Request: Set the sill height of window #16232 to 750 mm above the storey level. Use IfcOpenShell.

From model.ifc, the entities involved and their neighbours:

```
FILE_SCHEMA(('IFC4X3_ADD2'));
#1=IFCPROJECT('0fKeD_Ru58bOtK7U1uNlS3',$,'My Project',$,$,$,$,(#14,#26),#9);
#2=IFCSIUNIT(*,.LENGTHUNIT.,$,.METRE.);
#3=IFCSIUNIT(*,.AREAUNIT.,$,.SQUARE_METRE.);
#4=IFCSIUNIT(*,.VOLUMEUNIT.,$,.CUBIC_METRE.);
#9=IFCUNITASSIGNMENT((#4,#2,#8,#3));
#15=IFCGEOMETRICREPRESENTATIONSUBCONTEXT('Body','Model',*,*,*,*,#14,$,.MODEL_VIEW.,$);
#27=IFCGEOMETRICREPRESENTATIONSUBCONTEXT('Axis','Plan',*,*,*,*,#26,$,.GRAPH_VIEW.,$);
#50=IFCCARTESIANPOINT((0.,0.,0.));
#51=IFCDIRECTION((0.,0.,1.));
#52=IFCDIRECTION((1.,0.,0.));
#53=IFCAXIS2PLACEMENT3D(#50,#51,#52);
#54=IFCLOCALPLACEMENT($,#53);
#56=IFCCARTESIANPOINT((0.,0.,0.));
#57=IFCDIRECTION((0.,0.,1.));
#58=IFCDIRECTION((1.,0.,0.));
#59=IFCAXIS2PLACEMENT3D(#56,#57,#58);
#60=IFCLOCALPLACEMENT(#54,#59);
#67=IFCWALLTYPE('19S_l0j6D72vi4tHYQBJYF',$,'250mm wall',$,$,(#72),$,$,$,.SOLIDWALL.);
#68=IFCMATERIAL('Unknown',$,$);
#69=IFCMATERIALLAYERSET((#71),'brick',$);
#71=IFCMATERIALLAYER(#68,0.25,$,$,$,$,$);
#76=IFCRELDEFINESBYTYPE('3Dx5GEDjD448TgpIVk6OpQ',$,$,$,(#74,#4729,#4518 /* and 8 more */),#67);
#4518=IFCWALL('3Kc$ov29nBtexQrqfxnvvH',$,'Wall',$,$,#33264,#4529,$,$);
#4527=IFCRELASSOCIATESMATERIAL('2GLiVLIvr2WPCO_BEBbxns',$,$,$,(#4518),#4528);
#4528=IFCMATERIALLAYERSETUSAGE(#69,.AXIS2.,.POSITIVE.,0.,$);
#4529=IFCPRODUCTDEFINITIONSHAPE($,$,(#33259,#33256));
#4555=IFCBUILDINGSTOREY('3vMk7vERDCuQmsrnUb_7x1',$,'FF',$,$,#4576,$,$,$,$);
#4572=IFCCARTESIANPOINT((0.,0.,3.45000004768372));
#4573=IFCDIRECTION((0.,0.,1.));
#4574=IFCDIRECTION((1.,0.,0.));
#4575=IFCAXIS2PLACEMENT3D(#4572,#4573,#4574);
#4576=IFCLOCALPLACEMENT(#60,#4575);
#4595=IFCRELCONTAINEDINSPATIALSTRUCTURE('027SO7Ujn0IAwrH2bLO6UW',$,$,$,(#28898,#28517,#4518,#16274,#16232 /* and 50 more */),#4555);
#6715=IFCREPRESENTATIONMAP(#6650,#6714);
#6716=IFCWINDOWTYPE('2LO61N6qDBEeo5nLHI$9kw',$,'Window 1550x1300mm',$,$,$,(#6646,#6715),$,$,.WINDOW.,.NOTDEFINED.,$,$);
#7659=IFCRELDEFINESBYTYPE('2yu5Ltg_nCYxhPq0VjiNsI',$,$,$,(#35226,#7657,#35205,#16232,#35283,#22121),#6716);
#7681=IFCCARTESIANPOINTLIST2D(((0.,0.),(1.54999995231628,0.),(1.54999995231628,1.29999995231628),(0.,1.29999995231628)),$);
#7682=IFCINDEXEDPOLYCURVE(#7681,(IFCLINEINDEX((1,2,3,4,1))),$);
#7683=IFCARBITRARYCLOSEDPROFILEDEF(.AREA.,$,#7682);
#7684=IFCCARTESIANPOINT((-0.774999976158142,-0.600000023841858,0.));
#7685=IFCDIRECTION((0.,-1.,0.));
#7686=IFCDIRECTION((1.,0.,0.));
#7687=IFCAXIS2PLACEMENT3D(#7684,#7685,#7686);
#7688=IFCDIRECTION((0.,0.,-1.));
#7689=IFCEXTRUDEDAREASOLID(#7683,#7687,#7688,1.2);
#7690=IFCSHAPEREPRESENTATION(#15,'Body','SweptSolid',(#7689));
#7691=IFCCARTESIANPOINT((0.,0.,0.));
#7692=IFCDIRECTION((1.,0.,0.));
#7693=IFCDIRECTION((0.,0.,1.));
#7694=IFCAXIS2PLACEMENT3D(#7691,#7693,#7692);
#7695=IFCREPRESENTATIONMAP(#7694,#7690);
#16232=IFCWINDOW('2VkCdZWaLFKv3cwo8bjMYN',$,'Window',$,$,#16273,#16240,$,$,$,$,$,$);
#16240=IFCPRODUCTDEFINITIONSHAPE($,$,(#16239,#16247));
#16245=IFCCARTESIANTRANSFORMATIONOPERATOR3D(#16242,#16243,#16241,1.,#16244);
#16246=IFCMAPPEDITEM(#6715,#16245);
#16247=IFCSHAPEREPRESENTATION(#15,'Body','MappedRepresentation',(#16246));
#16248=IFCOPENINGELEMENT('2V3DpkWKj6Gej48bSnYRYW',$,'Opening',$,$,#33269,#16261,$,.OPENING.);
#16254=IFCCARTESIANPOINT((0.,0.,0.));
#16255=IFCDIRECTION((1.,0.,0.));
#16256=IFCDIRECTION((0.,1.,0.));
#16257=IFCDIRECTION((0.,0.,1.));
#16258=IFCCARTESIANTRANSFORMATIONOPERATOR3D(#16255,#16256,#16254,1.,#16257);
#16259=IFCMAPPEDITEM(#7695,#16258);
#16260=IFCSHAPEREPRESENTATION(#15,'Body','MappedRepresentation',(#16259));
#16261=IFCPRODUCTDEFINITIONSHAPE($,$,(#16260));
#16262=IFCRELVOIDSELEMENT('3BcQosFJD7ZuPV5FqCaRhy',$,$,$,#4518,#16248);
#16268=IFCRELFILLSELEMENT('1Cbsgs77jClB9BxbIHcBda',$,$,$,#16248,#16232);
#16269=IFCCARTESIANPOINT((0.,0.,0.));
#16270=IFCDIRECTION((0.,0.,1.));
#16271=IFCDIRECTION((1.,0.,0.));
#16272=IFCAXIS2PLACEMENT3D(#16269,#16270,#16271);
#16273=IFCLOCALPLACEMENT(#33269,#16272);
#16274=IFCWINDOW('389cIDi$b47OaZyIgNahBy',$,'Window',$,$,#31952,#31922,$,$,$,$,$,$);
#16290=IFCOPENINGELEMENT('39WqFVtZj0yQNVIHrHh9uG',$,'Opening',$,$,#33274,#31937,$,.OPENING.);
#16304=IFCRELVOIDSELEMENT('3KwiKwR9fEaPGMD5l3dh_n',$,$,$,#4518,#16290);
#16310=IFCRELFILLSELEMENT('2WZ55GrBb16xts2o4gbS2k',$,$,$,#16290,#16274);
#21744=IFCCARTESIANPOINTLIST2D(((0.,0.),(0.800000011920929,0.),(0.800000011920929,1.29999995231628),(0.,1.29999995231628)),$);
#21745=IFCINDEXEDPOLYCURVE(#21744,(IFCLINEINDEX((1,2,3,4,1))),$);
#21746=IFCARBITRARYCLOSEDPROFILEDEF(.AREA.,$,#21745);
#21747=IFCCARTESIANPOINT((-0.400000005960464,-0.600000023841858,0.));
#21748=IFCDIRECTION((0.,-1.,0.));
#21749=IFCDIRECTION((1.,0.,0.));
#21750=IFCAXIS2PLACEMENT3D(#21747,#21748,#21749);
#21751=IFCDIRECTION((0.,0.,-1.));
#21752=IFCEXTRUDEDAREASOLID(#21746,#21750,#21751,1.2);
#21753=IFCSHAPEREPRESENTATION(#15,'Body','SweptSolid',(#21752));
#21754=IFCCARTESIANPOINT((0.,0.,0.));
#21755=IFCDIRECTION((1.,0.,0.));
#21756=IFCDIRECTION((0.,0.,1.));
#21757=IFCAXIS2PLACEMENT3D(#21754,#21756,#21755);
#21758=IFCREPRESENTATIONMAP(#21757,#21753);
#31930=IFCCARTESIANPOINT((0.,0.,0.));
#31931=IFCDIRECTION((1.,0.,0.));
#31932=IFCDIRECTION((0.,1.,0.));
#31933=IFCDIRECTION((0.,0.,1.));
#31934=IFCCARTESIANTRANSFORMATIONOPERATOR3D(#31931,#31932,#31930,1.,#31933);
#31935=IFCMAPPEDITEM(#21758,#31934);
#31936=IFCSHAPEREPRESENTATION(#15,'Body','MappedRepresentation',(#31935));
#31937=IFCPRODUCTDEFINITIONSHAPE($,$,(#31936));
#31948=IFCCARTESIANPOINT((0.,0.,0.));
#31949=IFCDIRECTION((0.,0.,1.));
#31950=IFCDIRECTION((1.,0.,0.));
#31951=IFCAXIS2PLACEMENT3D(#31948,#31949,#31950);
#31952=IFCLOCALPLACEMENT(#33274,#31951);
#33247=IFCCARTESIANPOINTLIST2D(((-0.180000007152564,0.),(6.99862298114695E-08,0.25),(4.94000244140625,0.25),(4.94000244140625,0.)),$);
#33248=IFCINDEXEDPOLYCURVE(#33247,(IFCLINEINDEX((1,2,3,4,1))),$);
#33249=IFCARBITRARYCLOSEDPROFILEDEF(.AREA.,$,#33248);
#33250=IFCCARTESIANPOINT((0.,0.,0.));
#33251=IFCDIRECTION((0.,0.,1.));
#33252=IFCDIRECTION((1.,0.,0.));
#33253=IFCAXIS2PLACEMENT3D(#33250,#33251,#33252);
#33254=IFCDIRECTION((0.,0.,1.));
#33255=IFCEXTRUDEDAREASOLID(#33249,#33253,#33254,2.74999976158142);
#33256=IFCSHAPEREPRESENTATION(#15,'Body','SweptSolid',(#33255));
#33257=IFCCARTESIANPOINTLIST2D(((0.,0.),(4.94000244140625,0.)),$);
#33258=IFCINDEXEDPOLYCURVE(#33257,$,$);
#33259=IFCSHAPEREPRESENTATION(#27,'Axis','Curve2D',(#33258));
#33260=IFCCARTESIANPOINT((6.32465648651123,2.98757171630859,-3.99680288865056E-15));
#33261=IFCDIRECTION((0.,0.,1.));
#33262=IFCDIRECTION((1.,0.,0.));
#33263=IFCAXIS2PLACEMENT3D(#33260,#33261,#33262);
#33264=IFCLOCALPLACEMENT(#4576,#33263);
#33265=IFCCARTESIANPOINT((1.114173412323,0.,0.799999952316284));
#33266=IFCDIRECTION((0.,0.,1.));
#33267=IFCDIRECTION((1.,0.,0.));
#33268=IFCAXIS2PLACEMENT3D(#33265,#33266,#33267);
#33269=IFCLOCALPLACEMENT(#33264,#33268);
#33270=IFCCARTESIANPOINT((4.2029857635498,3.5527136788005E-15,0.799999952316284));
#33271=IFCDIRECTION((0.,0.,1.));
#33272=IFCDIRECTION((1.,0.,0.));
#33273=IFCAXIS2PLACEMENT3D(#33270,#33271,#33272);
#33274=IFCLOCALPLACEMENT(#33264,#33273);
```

```python
import numpy as np
import ifcopenshell
import ifcopenshell.api.geometry
import ifcopenshell.geom
import ifcopenshell.util.element
import ifcopenshell.util.placement
import ifcopenshell.util.shape
import ifcopenshell.util.unit

model = ifcopenshell.open("model.ifc")
unit_scale = ifcopenshell.util.unit.calculate_unit_scale(model)

window = model.by_guid("2VkCdZWaLFKv3cwo8bjMYN")
opening = window.FillsVoids[0].RelatingOpeningElement
storey = ifcopenshell.util.element.get_container(window, ifc_class="IfcBuildingStorey")
level = ifcopenshell.util.placement.get_local_placement(storey.ObjectPlacement)[2, 3]

# The opening's origin need not be at the sill, so measure its lowest point.
shape = ifcopenshell.geom.create_shape(ifcopenshell.geom.settings(), opening)
bottom = ifcopenshell.util.shape.get_shape_bottom_elevation(shape, shape.geometry) / unit_scale
dz = level + 0.75 / unit_scale - bottom

shift = np.array([0.0, 0.0, dz])
# The window is placed relative to its opening, so it follows when the opening moves.
matrix = ifcopenshell.util.placement.get_local_placement(opening.ObjectPlacement)
matrix[:3, 3] += shift
ifcopenshell.api.geometry.edit_object_placement(
    model, product=opening, matrix=matrix, is_si=False, should_transform_children=True
)

print(f"moved by {dz * unit_scale:+.3f} m")

model.write("model_updated.ifc")
```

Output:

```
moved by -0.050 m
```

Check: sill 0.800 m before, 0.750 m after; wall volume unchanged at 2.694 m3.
